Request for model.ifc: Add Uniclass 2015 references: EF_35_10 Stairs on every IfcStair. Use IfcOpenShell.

First a look at what the model holds.

```python
import ifcopenshell

model = ifcopenshell.open("model.ifc")
print(model.schema)
print("classifications:", [c.Name for c in model.by_type("IfcClassification")])
for ifc_class in ("IfcDoor", "IfcRoof", "IfcStair", "IfcWall", "IfcWindow"):
    print(ifc_class, len(model.by_type(ifc_class)))
```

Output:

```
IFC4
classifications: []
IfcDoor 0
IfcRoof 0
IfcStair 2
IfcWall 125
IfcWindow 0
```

```python
import ifcopenshell
import ifcopenshell.api.classification

model = ifcopenshell.open("model.ifc")

system = ifcopenshell.api.classification.add_classification(model, classification="Uniclass 2015")

codes = {
    "IfcStair": ("EF_35_10", "Stairs"),
}
for ifc_class, (code, name) in codes.items():
    products = model.by_type(ifc_class)
    ifcopenshell.api.classification.add_reference(
        model, products=products, classification=system, identification=code, name=name
    )
    print(code, len(products))

model.write("model_v2.ifc")
```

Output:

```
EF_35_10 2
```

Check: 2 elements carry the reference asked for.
